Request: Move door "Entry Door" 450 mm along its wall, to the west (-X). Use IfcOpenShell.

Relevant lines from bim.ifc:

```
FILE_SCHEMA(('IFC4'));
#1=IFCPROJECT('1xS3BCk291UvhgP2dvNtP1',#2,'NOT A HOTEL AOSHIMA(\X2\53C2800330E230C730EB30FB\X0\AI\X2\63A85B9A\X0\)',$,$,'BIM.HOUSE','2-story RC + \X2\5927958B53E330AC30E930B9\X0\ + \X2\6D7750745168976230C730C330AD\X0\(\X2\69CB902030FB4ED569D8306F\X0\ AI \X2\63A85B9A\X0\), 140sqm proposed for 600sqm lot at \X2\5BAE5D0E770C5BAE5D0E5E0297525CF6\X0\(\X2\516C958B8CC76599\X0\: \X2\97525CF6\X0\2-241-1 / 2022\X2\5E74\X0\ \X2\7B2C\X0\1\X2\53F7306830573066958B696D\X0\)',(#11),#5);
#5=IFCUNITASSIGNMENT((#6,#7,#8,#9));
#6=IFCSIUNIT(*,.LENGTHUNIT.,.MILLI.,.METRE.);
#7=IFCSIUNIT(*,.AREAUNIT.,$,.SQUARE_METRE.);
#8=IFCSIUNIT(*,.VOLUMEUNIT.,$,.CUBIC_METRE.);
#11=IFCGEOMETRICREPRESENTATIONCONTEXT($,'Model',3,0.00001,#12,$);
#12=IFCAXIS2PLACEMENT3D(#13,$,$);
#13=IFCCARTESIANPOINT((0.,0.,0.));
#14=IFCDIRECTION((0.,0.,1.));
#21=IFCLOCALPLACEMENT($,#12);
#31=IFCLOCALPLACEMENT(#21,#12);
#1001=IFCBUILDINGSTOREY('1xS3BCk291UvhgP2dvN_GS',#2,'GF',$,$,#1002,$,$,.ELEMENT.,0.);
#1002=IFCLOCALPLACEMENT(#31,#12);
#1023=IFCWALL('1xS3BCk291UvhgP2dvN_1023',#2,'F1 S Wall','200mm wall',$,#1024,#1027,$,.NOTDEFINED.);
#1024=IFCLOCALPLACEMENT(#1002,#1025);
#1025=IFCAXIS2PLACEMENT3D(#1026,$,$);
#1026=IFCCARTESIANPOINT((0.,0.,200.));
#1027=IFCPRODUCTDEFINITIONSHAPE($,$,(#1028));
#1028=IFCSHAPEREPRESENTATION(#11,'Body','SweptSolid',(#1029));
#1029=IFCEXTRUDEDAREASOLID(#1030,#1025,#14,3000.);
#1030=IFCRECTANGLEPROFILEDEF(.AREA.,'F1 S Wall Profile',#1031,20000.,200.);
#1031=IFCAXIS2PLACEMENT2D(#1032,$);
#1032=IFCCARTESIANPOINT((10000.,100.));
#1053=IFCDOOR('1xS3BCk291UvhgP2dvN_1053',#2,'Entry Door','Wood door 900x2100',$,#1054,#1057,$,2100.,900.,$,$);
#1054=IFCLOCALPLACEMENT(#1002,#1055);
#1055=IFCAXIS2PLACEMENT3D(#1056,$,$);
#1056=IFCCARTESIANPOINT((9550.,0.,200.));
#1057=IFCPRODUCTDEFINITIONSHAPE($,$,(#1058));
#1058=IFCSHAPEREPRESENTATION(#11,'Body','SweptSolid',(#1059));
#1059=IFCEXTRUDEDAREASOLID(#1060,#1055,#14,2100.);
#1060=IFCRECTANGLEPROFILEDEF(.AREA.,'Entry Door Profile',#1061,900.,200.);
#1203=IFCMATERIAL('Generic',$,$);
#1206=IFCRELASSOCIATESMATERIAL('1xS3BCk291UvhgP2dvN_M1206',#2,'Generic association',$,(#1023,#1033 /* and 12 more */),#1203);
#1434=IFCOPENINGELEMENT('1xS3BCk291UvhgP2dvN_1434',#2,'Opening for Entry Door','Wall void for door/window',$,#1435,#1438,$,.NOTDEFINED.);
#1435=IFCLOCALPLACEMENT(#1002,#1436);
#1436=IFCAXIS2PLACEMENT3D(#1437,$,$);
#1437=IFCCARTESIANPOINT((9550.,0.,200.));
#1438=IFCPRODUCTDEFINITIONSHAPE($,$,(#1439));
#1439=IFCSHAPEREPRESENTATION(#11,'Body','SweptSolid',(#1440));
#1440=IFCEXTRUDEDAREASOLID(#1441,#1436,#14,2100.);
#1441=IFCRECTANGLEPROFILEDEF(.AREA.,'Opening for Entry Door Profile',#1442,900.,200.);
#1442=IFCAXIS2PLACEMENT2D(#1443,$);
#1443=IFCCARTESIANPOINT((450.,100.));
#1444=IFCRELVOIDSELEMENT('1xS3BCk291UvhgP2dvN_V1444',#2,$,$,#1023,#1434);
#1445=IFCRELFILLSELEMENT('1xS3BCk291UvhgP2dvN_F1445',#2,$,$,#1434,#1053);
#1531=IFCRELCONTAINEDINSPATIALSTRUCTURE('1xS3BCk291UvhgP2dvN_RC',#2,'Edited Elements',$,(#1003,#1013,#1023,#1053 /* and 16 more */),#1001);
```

```python
import ifcopenshell
import ifcopenshell.api.geometry
import ifcopenshell.util.placement
import ifcopenshell.util.unit

model = ifcopenshell.open("bim.ifc")
unit_scale = ifcopenshell.util.unit.calculate_unit_scale(model)

door = model.by_guid("1xS3BCk291UvhgP2dvN_1053")
opening = door.FillsVoids[0].RelatingOpeningElement
wall = opening.VoidsElements[0].RelatingBuildingElement

wall_matrix = ifcopenshell.util.placement.get_local_placement(wall.ObjectPlacement)
shift = wall_matrix[:3, 0] * -0.45 / unit_scale
before = ifcopenshell.util.placement.get_local_placement(door.ObjectPlacement)[:3, 3].copy()

# The door is not placed relative to its opening, so move both.
for product in (opening, door):
    matrix = ifcopenshell.util.placement.get_local_placement(product.ObjectPlacement)
    matrix[:3, 3] += shift
    ifcopenshell.api.geometry.edit_object_placement(model, product=product, matrix=matrix, is_si=False)

after = ifcopenshell.util.placement.get_local_placement(door.ObjectPlacement)[:3, 3]
print("door moved by", (after - before).round(3) + 0.0)

model.write("bim-out.ifc")
```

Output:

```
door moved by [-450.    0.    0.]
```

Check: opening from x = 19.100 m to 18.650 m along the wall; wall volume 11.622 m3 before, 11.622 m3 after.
